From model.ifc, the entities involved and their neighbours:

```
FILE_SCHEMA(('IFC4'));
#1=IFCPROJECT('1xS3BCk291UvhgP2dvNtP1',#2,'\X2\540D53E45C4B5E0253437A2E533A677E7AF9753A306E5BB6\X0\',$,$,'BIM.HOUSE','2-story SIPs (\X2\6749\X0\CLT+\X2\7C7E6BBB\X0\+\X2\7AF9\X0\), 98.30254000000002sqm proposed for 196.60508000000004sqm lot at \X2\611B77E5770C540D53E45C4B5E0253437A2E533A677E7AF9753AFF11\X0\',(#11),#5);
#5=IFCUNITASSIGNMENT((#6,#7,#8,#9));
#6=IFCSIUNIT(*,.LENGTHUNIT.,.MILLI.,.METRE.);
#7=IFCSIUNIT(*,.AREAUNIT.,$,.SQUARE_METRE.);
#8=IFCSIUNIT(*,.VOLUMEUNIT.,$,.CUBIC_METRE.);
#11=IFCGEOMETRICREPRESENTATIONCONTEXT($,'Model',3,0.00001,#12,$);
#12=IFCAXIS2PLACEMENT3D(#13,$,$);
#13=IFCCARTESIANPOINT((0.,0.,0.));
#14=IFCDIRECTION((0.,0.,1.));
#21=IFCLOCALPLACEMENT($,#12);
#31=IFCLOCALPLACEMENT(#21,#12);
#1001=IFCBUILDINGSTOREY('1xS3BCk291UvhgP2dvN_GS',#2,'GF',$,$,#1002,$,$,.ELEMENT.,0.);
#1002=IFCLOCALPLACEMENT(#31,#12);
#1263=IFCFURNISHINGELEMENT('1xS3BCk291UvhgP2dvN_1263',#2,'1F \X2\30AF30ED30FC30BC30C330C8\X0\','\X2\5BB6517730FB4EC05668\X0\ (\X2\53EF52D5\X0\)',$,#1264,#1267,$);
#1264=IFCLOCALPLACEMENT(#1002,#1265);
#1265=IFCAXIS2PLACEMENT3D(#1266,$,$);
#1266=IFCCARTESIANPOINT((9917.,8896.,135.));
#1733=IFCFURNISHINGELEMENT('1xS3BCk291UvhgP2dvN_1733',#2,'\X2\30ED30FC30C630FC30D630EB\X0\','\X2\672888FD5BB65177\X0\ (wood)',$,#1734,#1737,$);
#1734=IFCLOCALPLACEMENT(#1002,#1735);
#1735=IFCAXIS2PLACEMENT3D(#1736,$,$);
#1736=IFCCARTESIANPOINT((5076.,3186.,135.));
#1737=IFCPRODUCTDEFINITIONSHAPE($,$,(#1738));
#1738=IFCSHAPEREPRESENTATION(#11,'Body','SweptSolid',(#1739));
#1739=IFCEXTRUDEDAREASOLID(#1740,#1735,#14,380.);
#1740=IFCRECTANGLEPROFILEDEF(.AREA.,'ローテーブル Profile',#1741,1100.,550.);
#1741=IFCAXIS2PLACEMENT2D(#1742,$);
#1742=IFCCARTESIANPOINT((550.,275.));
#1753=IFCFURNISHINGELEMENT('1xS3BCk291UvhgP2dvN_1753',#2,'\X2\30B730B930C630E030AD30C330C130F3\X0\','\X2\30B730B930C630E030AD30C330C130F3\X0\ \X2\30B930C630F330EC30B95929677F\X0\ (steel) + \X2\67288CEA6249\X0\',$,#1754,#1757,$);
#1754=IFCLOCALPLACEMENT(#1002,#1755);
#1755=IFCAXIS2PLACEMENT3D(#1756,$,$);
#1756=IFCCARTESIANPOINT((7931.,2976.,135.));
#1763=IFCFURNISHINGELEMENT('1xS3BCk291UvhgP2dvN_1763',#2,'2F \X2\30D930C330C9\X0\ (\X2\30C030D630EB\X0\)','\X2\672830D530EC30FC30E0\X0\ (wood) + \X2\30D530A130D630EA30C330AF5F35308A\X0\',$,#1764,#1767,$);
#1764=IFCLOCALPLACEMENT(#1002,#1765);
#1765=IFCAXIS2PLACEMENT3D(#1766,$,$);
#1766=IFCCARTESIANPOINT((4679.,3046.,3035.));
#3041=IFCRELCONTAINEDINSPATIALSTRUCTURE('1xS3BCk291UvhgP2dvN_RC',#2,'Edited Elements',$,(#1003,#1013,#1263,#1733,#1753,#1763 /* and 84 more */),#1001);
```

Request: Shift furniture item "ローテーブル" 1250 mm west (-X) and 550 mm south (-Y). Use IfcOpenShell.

```python
import ifcopenshell
import ifcopenshell.api.geometry
import ifcopenshell.util.placement
import ifcopenshell.util.unit

model = ifcopenshell.open("model.ifc")
unit_scale = ifcopenshell.util.unit.calculate_unit_scale(model)

item = model.by_guid("1xS3BCk291UvhgP2dvN_1733")
matrix = ifcopenshell.util.placement.get_local_placement(item.ObjectPlacement)
matrix[0, 3] -= 1.25 / unit_scale
matrix[1, 3] -= 0.55 / unit_scale
ifcopenshell.api.geometry.edit_object_placement(model, product=item, matrix=matrix, is_si=False)

print(ifcopenshell.util.placement.get_local_placement(item.ObjectPlacement).round(3) + 0.0)

model.write("model-out.ifc")
```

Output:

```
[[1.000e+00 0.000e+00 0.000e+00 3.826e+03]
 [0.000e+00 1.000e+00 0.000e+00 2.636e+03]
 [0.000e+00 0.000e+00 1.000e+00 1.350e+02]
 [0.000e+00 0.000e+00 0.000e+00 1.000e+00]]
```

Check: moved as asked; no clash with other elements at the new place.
